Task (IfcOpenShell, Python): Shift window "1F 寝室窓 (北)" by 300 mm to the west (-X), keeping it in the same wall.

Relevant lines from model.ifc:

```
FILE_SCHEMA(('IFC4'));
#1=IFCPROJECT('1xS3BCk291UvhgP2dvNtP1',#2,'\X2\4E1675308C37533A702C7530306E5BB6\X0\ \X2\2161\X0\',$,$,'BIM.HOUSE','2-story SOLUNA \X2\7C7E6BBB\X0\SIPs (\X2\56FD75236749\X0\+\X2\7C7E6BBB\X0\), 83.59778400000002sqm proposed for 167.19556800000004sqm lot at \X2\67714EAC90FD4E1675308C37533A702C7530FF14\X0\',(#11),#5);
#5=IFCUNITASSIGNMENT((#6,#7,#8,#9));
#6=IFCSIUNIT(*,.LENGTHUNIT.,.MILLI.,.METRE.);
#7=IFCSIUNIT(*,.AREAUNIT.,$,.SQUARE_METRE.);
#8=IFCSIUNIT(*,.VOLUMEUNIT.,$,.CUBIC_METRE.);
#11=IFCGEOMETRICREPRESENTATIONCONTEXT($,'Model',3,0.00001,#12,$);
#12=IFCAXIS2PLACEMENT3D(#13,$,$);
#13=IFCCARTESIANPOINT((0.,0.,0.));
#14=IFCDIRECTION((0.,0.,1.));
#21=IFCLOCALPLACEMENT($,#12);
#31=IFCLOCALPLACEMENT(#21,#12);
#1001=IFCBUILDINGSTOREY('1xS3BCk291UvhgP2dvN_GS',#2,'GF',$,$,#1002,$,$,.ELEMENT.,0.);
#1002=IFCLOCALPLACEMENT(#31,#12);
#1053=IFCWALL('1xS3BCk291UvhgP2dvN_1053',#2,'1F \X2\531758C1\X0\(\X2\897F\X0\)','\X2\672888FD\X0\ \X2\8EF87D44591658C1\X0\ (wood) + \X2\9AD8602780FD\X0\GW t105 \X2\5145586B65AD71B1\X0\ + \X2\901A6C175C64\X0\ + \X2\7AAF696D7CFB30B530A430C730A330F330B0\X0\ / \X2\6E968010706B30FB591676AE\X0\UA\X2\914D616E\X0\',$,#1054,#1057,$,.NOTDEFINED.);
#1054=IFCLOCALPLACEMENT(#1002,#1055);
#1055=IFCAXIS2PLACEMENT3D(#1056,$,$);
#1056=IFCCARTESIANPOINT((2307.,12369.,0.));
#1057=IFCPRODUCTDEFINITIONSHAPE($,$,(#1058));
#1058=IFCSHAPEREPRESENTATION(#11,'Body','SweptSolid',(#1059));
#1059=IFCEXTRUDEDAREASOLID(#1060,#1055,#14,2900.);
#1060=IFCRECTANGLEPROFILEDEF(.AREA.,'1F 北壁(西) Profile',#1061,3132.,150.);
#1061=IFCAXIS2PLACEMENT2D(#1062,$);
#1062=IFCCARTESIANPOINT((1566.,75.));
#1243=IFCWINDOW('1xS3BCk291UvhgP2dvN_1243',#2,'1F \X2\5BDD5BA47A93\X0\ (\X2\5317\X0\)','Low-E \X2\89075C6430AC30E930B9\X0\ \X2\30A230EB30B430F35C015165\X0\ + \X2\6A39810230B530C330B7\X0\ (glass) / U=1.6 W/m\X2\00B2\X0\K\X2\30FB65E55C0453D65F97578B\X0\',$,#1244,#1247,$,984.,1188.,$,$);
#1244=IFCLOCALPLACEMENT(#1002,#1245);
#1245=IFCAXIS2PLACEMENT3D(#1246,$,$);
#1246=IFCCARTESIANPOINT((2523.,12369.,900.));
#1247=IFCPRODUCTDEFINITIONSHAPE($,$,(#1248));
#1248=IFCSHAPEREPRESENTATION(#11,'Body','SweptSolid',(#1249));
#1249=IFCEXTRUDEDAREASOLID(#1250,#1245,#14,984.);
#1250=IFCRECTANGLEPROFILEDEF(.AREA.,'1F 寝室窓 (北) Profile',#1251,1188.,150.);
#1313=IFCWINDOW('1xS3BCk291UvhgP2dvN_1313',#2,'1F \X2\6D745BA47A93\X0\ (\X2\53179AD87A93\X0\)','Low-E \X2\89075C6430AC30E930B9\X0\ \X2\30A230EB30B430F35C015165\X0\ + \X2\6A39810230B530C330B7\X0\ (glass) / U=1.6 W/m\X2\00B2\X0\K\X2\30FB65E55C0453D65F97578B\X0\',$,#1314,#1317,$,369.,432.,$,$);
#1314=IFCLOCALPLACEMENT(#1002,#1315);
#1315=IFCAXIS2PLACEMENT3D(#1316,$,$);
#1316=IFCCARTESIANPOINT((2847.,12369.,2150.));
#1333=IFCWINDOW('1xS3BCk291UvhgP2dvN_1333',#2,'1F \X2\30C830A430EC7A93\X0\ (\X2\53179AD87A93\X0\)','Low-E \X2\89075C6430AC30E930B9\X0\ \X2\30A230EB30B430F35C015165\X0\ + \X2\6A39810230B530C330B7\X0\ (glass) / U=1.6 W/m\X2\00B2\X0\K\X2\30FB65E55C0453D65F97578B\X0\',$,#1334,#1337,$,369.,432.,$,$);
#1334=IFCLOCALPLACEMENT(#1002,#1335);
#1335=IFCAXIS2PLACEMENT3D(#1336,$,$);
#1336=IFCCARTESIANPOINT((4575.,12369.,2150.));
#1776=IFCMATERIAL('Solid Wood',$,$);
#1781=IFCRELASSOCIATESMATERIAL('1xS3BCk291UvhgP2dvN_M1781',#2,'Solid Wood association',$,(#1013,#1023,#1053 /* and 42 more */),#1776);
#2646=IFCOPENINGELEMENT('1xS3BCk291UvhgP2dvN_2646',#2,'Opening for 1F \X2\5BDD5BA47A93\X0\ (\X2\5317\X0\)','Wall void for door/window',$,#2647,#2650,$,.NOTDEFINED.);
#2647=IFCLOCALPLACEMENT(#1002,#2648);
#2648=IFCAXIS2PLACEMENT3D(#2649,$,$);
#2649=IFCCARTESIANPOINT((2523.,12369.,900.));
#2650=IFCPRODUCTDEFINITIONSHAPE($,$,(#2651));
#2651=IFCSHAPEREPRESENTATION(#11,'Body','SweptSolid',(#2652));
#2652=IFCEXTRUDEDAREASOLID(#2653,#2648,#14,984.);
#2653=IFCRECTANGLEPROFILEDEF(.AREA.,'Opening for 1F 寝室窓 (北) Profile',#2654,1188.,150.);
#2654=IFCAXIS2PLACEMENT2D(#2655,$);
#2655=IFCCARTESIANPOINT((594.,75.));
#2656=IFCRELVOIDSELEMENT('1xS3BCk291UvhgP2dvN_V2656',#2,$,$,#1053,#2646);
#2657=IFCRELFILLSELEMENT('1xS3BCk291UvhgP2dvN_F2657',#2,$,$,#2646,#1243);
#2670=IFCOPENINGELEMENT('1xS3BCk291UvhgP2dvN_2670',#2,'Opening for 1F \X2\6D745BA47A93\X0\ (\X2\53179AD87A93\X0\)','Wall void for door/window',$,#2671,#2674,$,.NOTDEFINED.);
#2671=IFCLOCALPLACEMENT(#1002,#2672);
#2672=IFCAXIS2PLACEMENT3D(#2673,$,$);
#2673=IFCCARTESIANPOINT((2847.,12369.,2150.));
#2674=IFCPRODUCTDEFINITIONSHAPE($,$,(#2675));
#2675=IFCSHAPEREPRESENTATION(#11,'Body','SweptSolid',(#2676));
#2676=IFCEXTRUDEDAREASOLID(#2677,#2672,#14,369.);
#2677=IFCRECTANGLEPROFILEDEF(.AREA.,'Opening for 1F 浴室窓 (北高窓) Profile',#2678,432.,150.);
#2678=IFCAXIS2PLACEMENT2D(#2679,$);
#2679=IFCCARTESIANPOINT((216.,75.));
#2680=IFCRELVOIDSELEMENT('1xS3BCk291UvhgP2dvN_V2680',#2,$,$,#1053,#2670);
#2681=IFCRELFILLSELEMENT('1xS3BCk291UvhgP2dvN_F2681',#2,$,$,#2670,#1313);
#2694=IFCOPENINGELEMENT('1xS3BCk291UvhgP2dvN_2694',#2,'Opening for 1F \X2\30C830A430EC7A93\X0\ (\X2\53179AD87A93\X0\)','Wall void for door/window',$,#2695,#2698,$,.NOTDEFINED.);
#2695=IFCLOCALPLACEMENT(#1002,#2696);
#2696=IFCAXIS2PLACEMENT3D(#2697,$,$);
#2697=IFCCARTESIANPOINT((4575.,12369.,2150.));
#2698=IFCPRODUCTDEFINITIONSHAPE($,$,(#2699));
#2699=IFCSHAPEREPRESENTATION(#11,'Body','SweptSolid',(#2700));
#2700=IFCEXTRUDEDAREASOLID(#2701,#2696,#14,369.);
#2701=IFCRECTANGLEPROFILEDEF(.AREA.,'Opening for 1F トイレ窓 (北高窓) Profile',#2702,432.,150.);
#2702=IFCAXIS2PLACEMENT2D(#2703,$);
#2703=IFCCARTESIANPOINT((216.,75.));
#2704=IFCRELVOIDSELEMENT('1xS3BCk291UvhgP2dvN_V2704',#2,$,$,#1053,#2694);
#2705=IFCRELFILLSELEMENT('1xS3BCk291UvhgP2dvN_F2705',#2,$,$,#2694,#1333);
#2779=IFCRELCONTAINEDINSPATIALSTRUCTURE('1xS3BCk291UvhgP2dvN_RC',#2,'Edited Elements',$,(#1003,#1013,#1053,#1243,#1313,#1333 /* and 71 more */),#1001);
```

```python
import ifcopenshell
import ifcopenshell.api.geometry
import ifcopenshell.util.placement

model = ifcopenshell.open("model.ifc")

window = model.by_guid("1xS3BCk291UvhgP2dvN_1243")
opening = window.FillsVoids[0].RelatingOpeningElement
wall = opening.VoidsElements[0].RelatingBuildingElement

wall_matrix = ifcopenshell.util.placement.get_local_placement(wall.ObjectPlacement)
shift = wall_matrix[:3, 0] * -300.0
before = ifcopenshell.util.placement.get_local_placement(window.ObjectPlacement)[:3, 3].copy()

# The window is not placed relative to its opening, so move both.
for product in (opening, window):
    matrix = ifcopenshell.util.placement.get_local_placement(product.ObjectPlacement)
    matrix[:3, 3] += shift
    ifcopenshell.api.geometry.edit_object_placement(model, product=product, matrix=matrix, is_si=False)

after = ifcopenshell.util.placement.get_local_placement(window.ObjectPlacement)[:3, 3]
print("window moved by", (after - before).round(3) + 0.0)

model.write("model_updated.ifc")
```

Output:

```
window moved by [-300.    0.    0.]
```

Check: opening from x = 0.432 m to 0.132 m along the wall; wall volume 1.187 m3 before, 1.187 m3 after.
